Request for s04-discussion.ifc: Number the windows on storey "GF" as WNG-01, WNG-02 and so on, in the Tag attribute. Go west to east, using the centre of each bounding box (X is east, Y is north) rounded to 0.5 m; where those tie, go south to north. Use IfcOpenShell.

First a look at what the model holds.

```python
import ifcopenshell
import ifcopenshell.util.element
import ifcopenshell.util.placement

model = ifcopenshell.open("s04-discussion.ifc")
print(model.schema)
storey = next(s for s in model.by_type("IfcBuildingStorey") if s.Name == "GF")
windows = [e for e in ifcopenshell.util.element.get_decomposition(storey) if e.is_a("IfcWindow")]
for e in sorted(windows, key=lambda e: e.id()):
    origin = ifcopenshell.util.placement.get_local_placement(e.ObjectPlacement)[:3, 3]
    print(e.id(), e.Tag, e.Name, origin.round(2) + 0.0, sep=" | ")
```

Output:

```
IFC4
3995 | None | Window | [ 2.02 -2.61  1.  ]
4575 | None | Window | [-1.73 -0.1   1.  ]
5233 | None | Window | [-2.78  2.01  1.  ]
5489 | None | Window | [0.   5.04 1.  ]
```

```python
import ifcopenshell
import ifcopenshell.geom
import ifcopenshell.util.element
import ifcopenshell.util.shape

model = ifcopenshell.open("s04-discussion.ifc")
settings = ifcopenshell.geom.settings()
settings.set("use-world-coords", True)


def centre(element):
    shape = ifcopenshell.geom.create_shape(settings, element)
    return ifcopenshell.util.shape.get_bbox_centroid(shape.geometry)


storey = next(s for s in model.by_type("IfcBuildingStorey") if s.Name == "GF")
windows = [e for e in ifcopenshell.util.element.get_decomposition(storey) if e.is_a("IfcWindow")]

# Insertion points can sit at a corner or the storey origin, so sort by the geometry (in metres).
centres = {e: centre(e) for e in windows}
windows.sort(key=lambda e: (round(centres[e][0] / 0.5), centres[e][1]))

for i, e in enumerate(windows, start=1):
    number = f"WNG-{i:02d}"
    e.Tag = number
    print(e.id(), number)

model.write("s04-discussion_rev.ifc")
```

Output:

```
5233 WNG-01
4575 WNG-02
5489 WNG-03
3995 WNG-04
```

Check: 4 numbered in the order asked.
